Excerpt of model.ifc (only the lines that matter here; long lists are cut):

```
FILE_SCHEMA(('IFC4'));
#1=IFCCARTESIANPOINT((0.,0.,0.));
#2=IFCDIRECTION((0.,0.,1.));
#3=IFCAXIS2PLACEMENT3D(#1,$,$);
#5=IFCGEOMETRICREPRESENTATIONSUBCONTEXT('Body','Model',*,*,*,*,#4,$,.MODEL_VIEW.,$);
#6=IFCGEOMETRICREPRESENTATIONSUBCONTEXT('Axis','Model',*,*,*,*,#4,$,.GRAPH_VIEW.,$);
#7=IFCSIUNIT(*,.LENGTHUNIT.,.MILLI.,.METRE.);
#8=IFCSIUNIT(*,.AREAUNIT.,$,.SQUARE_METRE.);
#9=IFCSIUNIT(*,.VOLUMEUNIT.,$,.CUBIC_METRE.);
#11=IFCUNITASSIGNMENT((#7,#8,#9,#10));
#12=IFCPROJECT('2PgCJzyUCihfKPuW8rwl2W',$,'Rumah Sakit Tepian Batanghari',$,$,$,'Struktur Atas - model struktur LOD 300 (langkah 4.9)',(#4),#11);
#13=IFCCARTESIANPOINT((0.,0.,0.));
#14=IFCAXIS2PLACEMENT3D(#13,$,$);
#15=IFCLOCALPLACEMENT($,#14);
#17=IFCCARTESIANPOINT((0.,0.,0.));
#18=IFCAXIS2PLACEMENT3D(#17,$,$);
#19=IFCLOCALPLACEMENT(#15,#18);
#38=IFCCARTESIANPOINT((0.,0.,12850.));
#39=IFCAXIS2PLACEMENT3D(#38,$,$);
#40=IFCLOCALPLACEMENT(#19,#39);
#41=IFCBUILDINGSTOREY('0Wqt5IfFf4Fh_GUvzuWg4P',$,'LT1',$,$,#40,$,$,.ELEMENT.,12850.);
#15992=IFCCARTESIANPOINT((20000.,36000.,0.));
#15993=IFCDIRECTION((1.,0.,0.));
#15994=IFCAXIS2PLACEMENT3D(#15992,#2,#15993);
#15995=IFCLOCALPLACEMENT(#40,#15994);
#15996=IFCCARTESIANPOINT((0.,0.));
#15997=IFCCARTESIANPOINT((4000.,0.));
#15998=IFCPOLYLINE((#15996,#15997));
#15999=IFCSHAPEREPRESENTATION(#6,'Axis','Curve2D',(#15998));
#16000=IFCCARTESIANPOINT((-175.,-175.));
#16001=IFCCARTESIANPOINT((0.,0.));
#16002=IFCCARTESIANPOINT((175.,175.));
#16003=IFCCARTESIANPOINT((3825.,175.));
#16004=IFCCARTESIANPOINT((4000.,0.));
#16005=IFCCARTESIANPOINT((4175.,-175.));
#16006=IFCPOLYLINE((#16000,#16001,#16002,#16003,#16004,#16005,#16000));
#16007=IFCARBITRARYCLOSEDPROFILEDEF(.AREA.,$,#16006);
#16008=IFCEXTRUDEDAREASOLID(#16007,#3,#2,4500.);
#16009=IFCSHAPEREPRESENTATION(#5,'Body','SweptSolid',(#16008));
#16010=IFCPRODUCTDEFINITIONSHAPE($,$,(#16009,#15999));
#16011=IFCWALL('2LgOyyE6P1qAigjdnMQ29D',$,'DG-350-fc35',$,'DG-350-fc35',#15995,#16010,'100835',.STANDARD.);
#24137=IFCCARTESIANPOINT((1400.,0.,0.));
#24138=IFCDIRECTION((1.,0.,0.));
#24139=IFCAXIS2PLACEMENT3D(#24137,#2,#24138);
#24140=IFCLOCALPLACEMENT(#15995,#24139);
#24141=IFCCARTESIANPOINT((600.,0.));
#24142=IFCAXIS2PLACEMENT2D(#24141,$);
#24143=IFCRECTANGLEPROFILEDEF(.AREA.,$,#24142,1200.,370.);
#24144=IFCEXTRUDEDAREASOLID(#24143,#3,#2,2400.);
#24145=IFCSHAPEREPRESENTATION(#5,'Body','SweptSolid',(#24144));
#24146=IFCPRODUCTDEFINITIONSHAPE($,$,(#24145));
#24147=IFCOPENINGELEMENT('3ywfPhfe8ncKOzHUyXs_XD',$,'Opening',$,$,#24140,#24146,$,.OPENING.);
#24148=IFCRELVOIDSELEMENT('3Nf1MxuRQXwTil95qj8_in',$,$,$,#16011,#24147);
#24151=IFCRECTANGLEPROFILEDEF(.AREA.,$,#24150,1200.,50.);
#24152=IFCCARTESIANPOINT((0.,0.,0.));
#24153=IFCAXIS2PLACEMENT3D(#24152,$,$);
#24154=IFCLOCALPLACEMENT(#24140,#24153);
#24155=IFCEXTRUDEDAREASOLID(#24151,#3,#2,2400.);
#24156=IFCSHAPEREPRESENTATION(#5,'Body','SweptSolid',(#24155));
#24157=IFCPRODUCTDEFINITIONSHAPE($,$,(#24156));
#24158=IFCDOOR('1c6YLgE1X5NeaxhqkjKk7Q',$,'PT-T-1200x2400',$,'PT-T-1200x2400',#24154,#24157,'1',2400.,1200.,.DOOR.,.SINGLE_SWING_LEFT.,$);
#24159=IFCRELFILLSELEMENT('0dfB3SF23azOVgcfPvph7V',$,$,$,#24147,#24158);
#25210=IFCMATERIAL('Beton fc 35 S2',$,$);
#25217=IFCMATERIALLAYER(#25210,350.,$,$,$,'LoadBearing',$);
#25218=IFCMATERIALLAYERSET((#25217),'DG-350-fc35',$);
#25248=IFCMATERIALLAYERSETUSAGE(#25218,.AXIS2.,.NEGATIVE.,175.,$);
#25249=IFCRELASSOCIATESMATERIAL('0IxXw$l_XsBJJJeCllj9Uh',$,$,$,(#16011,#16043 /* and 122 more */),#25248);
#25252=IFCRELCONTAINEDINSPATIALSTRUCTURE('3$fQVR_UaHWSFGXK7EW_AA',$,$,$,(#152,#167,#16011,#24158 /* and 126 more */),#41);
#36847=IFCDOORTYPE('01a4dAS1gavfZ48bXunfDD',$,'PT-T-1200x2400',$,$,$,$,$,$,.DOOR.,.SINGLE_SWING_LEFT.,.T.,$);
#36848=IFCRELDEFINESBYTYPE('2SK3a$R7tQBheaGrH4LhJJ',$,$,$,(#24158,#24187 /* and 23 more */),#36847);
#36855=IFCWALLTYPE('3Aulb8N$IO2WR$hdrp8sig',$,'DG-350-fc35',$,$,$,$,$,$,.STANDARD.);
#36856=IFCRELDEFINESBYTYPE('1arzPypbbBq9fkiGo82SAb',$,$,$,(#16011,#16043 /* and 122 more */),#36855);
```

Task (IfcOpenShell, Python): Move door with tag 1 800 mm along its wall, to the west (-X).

```python
import ifcopenshell
import ifcopenshell.api.geometry
import ifcopenshell.util.placement
import ifcopenshell.util.unit

model = ifcopenshell.open("model.ifc")
unit_scale = ifcopenshell.util.unit.calculate_unit_scale(model)

door = model.by_guid("1c6YLgE1X5NeaxhqkjKk7Q")
opening = door.FillsVoids[0].RelatingOpeningElement
wall = opening.VoidsElements[0].RelatingBuildingElement

wall_matrix = ifcopenshell.util.placement.get_local_placement(wall.ObjectPlacement)
shift = wall_matrix[:3, 0] * -0.8 / unit_scale
before = ifcopenshell.util.placement.get_local_placement(door.ObjectPlacement)[:3, 3].copy()

# The door is placed relative to its opening, so it follows when the opening moves.
matrix = ifcopenshell.util.placement.get_local_placement(opening.ObjectPlacement)
matrix[:3, 3] += shift
ifcopenshell.api.geometry.edit_object_placement(
    model, product=opening, matrix=matrix, is_si=False, should_transform_children=True
)

after = ifcopenshell.util.placement.get_local_placement(door.ObjectPlacement)[:3, 3]
print("door moved by", (after - before).round(3) + 0.0)

model.write("model_v2.ifc")
```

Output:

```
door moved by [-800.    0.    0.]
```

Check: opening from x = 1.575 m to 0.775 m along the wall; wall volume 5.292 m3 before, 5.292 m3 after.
